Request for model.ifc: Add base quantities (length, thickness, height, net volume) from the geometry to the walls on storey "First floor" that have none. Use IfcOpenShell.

First a look at what the model holds.

```python
import ifcopenshell
import ifcopenshell.util.element
import ifcopenshell.util.unit

model = ifcopenshell.open("model.ifc")
print(model.schema)
for unit_type in ("LENGTHUNIT", "AREAUNIT", "VOLUMEUNIT"):
    print(unit_type, ifcopenshell.util.unit.calculate_unit_scale(model, unit_type))
storey = next(s for s in model.by_type("IfcBuildingStorey") if s.Name == "First floor")
walls = [e for e in ifcopenshell.util.element.get_decomposition(storey) if e.is_a("IfcWall")]
for e in sorted(walls, key=lambda e: e.id()):
    print(e.id(), e.is_a(), e.Name, list(ifcopenshell.util.element.get_psets(e, qtos_only=True)), sep=" | ")
```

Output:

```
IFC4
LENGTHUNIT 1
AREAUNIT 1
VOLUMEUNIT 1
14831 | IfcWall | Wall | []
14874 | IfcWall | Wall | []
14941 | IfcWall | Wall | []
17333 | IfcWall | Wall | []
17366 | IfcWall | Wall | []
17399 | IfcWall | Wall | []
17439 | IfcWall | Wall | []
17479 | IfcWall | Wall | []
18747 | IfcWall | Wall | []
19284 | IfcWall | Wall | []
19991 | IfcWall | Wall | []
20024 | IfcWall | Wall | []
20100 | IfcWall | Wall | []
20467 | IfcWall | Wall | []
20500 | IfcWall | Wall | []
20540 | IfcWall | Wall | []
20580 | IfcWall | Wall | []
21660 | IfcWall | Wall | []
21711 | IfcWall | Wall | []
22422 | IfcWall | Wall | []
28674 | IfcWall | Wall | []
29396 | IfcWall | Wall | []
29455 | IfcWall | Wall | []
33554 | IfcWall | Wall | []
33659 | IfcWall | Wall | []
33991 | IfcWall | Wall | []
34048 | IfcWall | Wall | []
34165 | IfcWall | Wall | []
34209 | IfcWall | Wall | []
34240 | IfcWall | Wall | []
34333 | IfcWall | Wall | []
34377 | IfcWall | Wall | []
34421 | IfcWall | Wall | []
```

```python
import ifcopenshell
import ifcopenshell.api.pset
import ifcopenshell.geom
import ifcopenshell.util.element
import ifcopenshell.util.shape
import ifcopenshell.util.unit

model = ifcopenshell.open("model.ifc")
unit_scale = ifcopenshell.util.unit.calculate_unit_scale(model)
volume_scale = ifcopenshell.util.unit.calculate_unit_scale(model, "VOLUMEUNIT")
settings = ifcopenshell.geom.settings()

storey = next(s for s in model.by_type("IfcBuildingStorey") if s.Name == "First floor")
walls = [e for e in ifcopenshell.util.element.get_decomposition(storey) if e.is_a("IfcWall")]

for e in sorted(walls, key=lambda e: e.id()):
    if ifcopenshell.util.element.get_psets(e, qtos_only=True, should_inherit=False):
        continue
    # Geometry comes back in metres, in the element's own axes.
    shape = ifcopenshell.geom.create_shape(settings, e)
    values = {
        "Length": ifcopenshell.util.shape.get_x(shape.geometry) / unit_scale,
        "Width": ifcopenshell.util.shape.get_y(shape.geometry) / unit_scale,
        "Height": ifcopenshell.util.shape.get_z(shape.geometry) / unit_scale,
        "NetVolume": ifcopenshell.util.shape.get_volume(shape.geometry) / volume_scale,
    }
    qto = ifcopenshell.api.pset.add_qto(model, product=e, name="Qto_WallBaseQuantities")
    ifcopenshell.api.pset.edit_qto(model, qto=qto, properties=values)
    print(e.id(), {k: round(v, 3) for k, v in values.items()})

model.write("model_edited.ifc")
```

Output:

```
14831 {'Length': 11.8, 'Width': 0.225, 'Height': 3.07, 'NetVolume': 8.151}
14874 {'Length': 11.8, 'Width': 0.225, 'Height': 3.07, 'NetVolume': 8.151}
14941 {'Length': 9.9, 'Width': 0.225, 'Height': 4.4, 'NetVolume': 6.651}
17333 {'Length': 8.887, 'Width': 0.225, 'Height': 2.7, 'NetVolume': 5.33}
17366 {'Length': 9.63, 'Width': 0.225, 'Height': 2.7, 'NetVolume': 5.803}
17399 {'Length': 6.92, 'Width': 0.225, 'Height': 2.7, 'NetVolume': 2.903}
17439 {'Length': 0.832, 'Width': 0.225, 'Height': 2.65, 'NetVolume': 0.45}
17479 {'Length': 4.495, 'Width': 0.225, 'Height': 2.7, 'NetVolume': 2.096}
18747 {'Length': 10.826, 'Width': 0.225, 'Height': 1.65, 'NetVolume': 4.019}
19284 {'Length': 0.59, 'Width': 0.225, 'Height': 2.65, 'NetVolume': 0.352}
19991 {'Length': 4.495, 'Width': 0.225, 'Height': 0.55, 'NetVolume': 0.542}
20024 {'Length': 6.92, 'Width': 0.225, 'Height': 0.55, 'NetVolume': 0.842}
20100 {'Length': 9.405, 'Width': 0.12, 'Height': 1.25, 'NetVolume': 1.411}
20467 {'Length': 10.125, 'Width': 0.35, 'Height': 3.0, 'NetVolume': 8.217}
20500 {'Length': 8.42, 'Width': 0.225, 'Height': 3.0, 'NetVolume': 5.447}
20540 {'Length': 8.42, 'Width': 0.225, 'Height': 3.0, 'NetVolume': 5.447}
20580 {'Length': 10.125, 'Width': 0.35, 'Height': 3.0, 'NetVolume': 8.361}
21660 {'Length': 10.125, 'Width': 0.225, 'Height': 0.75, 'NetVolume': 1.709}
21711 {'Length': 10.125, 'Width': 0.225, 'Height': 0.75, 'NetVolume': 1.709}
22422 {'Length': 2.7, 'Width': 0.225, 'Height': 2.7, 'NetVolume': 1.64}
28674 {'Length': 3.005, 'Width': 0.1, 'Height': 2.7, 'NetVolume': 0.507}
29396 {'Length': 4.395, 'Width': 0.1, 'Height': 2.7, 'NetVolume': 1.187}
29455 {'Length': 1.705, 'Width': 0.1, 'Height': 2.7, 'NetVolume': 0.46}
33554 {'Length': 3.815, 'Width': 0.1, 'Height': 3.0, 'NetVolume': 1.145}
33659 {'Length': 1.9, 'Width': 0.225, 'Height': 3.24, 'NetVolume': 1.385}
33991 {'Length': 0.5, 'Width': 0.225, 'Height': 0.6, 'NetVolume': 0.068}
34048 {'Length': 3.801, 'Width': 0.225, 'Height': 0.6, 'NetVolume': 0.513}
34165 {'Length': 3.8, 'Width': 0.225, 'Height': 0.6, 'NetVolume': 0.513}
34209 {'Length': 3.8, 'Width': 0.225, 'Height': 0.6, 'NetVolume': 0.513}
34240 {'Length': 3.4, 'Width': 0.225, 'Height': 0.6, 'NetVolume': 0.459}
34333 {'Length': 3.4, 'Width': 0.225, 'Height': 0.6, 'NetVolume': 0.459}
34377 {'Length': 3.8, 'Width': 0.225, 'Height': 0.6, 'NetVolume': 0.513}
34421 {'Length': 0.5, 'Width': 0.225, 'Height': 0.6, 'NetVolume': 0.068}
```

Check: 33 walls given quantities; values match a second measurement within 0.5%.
